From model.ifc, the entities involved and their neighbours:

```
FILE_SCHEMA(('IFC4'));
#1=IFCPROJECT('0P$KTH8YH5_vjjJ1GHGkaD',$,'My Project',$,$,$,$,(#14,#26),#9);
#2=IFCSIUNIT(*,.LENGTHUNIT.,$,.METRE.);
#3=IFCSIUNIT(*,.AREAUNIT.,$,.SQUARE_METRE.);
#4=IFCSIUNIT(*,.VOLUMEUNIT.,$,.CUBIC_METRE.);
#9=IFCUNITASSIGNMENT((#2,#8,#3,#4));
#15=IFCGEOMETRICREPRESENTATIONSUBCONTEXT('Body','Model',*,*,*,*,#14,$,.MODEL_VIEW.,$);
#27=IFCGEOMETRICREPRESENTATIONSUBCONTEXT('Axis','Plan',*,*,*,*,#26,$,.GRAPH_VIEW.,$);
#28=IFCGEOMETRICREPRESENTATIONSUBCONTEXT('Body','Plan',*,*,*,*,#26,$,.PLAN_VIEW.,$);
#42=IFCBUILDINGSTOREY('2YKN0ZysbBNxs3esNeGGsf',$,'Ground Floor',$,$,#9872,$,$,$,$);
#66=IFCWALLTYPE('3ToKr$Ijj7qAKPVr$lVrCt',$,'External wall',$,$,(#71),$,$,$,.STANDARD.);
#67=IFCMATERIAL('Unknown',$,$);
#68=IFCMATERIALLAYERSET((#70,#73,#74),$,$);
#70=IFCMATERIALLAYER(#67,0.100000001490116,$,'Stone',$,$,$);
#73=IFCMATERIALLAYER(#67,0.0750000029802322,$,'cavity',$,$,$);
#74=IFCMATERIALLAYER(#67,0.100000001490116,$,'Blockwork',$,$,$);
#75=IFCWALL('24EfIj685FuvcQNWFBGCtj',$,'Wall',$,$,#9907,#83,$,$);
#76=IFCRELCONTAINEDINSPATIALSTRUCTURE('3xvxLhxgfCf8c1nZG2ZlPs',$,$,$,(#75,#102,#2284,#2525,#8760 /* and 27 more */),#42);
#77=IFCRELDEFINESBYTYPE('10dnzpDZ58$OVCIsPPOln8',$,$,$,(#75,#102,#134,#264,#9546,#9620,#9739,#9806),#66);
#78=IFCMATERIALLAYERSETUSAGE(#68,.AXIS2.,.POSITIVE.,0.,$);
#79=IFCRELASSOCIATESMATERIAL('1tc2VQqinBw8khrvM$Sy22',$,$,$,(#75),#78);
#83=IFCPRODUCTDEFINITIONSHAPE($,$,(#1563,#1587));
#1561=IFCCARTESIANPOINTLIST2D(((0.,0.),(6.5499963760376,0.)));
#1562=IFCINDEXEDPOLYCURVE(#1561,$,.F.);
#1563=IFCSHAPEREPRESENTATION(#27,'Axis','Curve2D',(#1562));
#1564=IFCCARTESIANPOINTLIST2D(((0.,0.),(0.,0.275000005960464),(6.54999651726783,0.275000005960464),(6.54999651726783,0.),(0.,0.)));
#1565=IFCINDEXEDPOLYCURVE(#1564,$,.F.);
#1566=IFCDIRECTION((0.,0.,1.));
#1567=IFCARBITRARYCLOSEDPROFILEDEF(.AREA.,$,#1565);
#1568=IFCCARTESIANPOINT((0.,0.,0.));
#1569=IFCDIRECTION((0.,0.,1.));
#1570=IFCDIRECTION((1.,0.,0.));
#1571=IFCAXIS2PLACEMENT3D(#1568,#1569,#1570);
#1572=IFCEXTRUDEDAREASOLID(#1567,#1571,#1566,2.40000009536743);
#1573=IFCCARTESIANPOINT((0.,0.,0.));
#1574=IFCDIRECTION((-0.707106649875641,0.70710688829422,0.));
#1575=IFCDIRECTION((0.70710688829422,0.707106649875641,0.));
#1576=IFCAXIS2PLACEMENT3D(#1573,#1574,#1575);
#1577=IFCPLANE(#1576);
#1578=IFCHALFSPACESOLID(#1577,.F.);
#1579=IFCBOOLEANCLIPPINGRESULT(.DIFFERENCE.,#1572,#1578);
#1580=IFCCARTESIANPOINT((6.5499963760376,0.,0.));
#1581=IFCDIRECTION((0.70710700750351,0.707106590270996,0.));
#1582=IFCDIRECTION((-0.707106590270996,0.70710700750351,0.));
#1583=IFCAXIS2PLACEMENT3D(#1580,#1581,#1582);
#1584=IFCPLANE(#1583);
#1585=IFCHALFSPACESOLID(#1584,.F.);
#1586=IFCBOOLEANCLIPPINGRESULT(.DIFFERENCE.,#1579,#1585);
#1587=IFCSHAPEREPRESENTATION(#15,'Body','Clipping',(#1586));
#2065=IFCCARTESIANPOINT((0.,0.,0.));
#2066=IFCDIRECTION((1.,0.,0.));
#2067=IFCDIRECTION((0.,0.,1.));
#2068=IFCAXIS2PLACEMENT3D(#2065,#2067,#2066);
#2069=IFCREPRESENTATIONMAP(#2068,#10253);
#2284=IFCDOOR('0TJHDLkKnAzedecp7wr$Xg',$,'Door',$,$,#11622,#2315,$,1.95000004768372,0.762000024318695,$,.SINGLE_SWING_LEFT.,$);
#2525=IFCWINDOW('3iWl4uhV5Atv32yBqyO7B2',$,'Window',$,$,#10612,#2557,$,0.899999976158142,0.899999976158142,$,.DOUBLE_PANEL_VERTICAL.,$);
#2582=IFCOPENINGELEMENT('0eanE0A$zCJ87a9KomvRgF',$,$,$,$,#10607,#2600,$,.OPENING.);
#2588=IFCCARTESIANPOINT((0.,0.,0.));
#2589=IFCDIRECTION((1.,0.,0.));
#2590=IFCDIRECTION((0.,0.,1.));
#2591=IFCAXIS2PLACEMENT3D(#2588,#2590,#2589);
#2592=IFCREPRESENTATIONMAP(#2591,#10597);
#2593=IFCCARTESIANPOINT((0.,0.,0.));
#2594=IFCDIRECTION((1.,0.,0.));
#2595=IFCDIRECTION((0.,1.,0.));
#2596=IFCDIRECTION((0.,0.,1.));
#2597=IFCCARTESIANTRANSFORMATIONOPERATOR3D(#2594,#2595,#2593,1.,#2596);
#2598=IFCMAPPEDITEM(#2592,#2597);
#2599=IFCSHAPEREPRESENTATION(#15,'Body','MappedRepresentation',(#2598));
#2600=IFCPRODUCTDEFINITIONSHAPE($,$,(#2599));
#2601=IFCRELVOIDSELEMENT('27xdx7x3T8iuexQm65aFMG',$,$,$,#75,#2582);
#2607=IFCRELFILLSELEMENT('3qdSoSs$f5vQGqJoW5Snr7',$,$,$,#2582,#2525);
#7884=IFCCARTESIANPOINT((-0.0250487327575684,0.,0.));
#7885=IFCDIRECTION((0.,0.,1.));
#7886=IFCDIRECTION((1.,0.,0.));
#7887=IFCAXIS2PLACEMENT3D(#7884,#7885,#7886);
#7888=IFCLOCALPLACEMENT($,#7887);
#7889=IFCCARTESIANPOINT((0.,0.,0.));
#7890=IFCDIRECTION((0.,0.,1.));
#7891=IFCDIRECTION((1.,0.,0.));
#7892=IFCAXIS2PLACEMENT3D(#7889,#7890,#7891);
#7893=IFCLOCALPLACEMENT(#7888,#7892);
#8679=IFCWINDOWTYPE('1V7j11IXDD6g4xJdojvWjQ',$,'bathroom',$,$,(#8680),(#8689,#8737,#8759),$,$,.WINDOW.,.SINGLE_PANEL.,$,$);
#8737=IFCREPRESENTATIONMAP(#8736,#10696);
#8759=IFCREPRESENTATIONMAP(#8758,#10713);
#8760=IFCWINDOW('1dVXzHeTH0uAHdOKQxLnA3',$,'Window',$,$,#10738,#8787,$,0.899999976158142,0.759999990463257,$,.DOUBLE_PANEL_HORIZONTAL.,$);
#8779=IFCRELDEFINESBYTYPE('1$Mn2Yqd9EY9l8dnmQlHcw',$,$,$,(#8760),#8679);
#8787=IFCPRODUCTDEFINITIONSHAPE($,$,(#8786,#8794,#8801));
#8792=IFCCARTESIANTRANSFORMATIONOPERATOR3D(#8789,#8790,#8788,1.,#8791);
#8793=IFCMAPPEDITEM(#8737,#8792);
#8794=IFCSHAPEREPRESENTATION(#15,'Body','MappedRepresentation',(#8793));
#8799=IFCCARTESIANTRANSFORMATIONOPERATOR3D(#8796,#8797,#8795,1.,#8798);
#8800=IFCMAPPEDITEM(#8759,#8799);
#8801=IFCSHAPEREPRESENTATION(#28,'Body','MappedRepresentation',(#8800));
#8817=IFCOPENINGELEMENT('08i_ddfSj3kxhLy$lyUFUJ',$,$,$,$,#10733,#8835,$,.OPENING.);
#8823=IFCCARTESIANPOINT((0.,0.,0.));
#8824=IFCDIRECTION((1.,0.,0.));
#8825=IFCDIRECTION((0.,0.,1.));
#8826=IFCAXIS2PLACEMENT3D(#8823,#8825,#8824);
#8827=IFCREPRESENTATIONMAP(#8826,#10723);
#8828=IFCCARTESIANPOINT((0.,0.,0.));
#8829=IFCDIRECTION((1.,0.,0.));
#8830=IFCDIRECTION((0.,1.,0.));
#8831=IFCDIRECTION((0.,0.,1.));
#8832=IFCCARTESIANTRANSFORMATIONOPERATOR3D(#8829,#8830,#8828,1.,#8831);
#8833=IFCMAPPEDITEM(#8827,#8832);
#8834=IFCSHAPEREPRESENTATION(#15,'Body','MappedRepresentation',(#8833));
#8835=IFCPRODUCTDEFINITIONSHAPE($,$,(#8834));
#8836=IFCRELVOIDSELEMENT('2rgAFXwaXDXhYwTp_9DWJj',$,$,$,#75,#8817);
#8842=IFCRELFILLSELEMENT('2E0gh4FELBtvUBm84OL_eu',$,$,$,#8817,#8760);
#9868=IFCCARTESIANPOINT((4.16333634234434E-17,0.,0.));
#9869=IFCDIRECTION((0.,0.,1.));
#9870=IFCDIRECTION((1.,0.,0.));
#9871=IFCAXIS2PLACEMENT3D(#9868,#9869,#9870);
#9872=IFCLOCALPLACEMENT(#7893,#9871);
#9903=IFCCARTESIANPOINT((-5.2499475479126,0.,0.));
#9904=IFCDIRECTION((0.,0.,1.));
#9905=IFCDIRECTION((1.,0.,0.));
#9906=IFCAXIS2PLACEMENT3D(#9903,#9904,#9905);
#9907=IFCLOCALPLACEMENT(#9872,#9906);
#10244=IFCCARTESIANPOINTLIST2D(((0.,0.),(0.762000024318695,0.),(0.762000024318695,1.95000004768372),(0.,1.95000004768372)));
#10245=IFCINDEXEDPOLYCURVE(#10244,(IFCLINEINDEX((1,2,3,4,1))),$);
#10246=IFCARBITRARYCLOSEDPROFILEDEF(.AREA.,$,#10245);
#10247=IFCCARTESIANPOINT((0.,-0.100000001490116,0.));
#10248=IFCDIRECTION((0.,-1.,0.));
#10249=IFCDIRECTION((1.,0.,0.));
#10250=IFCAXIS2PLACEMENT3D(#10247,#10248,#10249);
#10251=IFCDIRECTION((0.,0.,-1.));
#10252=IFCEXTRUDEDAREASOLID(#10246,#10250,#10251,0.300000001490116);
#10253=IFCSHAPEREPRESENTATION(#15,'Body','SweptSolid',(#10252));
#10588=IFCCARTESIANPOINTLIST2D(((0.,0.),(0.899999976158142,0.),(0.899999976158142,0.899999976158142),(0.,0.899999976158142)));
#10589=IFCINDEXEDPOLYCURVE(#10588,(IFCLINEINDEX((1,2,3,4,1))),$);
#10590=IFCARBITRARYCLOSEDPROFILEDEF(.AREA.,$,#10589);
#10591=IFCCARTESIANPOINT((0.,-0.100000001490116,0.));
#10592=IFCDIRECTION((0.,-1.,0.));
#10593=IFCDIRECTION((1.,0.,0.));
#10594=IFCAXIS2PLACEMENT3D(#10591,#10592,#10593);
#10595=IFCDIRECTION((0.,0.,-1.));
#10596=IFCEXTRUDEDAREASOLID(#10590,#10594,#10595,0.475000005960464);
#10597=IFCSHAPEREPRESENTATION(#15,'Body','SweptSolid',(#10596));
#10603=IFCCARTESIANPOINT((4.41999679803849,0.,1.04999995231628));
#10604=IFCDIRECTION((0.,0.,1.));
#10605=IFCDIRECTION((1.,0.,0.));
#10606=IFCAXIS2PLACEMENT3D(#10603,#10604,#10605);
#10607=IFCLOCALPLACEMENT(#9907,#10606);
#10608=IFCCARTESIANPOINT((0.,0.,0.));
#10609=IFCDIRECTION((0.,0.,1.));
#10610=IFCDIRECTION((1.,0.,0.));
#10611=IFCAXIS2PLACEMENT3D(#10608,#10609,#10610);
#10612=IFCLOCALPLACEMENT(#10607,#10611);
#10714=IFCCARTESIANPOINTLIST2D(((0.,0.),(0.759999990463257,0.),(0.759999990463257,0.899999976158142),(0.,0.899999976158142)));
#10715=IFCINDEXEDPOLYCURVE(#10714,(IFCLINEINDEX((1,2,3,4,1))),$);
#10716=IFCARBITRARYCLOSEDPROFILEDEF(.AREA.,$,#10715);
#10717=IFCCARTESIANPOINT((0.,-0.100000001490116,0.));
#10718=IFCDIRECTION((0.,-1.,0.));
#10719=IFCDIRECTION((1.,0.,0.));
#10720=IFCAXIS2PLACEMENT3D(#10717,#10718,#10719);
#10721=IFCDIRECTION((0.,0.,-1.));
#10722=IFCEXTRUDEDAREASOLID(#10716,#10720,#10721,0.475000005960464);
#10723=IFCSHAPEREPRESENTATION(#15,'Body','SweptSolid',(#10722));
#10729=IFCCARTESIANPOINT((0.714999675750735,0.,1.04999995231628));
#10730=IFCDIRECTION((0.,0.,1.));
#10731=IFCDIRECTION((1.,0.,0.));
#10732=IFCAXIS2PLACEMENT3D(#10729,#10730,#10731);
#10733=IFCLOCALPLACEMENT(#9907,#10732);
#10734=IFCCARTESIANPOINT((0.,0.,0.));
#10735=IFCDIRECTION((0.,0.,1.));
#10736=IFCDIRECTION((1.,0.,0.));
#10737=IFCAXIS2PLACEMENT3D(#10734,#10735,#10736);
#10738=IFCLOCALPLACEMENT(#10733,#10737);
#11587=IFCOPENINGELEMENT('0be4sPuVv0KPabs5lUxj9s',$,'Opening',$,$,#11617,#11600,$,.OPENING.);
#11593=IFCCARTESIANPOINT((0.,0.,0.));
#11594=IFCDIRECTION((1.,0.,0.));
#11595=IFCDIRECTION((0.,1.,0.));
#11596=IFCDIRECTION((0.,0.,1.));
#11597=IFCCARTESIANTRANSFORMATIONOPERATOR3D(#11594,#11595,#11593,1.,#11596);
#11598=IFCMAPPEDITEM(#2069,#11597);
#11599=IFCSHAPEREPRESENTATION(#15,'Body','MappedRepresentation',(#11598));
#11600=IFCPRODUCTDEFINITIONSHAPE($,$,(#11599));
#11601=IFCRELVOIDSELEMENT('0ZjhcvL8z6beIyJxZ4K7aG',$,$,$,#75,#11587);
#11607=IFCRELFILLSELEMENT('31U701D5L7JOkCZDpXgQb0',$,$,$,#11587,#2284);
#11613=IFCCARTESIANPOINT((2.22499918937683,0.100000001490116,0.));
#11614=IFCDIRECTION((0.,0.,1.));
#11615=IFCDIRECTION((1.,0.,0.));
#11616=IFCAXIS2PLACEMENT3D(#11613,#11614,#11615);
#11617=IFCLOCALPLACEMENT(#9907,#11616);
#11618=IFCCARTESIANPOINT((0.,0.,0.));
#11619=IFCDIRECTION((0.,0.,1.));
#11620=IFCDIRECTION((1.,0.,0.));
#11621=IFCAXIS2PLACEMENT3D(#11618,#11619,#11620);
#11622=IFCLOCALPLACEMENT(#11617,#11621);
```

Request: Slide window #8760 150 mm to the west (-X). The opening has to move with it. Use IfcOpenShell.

```python
import ifcopenshell
import ifcopenshell.api.geometry
import ifcopenshell.util.placement

model = ifcopenshell.open("model.ifc")

window = model.by_guid("1dVXzHeTH0uAHdOKQxLnA3")
opening = window.FillsVoids[0].RelatingOpeningElement
wall = opening.VoidsElements[0].RelatingBuildingElement

wall_matrix = ifcopenshell.util.placement.get_local_placement(wall.ObjectPlacement)
shift = wall_matrix[:3, 0] * -0.15
before = ifcopenshell.util.placement.get_local_placement(window.ObjectPlacement)[:3, 3].copy()

# The window is placed relative to its opening, so it follows when the opening moves.
matrix = ifcopenshell.util.placement.get_local_placement(opening.ObjectPlacement)
matrix[:3, 3] += shift
ifcopenshell.api.geometry.edit_object_placement(
    model, product=opening, matrix=matrix, is_si=False, should_transform_children=True
)

after = ifcopenshell.util.placement.get_local_placement(window.ObjectPlacement)[:3, 3]
print("window moved by", (after - before).round(3) + 0.0)

model.write("model_rev.ifc")
```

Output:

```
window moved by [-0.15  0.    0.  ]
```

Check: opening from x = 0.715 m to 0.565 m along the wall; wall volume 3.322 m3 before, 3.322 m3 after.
